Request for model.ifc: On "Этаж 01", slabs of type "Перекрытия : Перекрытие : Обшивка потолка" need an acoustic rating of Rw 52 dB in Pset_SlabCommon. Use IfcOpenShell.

First a look at what the model holds.

```python
import ifcopenshell
import ifcopenshell.util.element

model = ifcopenshell.open("model.ifc")
print(model.schema)
storey = next(s for s in model.by_type("IfcBuildingStorey") if s.Name == "Этаж 01")
slabs = [e for e in ifcopenshell.util.element.get_decomposition(storey) if e.is_a("IfcSlab")]
seen = {}
for e in slabs:
    element_type = ifcopenshell.util.element.get_type(e)
    key = (element_type.Name if element_type != e and element_type else None, ifcopenshell.util.element.get_pset(e, "Pset_SlabCommon", "AcousticRating"))
    seen[key] = seen.get(key, 0) + 1
for (name, value), count in sorted(seen.items(), key=str):
    print(count, "x", name, "|", value)
```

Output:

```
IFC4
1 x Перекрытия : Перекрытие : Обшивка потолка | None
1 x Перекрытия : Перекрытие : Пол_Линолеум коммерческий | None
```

```python
import ifcopenshell
import ifcopenshell.api.pset
import ifcopenshell.util.element

model = ifcopenshell.open("model.ifc")

storey = next(s for s in model.by_type("IfcBuildingStorey") if s.Name == "Этаж 01")
slabs = [e for e in ifcopenshell.util.element.get_decomposition(storey) if e.is_a("IfcSlab")]

count = 0
for e in slabs:
    element_type = ifcopenshell.util.element.get_type(e)
    if element_type in (None, e) or element_type.Name != "Перекрытия : Перекрытие : Обшивка потолка":
        continue
    # add_pset returns the element's existing set when there is one.
    pset = ifcopenshell.api.pset.add_pset(model, product=e, name="Pset_SlabCommon")
    ifcopenshell.api.pset.edit_pset(model, pset=pset, properties={"AcousticRating": "Rw 52 dB"})
    count += 1

print(count, "slabs updated")

model.write("model_rev.ifc")
```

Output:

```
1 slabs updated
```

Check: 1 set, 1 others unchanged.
